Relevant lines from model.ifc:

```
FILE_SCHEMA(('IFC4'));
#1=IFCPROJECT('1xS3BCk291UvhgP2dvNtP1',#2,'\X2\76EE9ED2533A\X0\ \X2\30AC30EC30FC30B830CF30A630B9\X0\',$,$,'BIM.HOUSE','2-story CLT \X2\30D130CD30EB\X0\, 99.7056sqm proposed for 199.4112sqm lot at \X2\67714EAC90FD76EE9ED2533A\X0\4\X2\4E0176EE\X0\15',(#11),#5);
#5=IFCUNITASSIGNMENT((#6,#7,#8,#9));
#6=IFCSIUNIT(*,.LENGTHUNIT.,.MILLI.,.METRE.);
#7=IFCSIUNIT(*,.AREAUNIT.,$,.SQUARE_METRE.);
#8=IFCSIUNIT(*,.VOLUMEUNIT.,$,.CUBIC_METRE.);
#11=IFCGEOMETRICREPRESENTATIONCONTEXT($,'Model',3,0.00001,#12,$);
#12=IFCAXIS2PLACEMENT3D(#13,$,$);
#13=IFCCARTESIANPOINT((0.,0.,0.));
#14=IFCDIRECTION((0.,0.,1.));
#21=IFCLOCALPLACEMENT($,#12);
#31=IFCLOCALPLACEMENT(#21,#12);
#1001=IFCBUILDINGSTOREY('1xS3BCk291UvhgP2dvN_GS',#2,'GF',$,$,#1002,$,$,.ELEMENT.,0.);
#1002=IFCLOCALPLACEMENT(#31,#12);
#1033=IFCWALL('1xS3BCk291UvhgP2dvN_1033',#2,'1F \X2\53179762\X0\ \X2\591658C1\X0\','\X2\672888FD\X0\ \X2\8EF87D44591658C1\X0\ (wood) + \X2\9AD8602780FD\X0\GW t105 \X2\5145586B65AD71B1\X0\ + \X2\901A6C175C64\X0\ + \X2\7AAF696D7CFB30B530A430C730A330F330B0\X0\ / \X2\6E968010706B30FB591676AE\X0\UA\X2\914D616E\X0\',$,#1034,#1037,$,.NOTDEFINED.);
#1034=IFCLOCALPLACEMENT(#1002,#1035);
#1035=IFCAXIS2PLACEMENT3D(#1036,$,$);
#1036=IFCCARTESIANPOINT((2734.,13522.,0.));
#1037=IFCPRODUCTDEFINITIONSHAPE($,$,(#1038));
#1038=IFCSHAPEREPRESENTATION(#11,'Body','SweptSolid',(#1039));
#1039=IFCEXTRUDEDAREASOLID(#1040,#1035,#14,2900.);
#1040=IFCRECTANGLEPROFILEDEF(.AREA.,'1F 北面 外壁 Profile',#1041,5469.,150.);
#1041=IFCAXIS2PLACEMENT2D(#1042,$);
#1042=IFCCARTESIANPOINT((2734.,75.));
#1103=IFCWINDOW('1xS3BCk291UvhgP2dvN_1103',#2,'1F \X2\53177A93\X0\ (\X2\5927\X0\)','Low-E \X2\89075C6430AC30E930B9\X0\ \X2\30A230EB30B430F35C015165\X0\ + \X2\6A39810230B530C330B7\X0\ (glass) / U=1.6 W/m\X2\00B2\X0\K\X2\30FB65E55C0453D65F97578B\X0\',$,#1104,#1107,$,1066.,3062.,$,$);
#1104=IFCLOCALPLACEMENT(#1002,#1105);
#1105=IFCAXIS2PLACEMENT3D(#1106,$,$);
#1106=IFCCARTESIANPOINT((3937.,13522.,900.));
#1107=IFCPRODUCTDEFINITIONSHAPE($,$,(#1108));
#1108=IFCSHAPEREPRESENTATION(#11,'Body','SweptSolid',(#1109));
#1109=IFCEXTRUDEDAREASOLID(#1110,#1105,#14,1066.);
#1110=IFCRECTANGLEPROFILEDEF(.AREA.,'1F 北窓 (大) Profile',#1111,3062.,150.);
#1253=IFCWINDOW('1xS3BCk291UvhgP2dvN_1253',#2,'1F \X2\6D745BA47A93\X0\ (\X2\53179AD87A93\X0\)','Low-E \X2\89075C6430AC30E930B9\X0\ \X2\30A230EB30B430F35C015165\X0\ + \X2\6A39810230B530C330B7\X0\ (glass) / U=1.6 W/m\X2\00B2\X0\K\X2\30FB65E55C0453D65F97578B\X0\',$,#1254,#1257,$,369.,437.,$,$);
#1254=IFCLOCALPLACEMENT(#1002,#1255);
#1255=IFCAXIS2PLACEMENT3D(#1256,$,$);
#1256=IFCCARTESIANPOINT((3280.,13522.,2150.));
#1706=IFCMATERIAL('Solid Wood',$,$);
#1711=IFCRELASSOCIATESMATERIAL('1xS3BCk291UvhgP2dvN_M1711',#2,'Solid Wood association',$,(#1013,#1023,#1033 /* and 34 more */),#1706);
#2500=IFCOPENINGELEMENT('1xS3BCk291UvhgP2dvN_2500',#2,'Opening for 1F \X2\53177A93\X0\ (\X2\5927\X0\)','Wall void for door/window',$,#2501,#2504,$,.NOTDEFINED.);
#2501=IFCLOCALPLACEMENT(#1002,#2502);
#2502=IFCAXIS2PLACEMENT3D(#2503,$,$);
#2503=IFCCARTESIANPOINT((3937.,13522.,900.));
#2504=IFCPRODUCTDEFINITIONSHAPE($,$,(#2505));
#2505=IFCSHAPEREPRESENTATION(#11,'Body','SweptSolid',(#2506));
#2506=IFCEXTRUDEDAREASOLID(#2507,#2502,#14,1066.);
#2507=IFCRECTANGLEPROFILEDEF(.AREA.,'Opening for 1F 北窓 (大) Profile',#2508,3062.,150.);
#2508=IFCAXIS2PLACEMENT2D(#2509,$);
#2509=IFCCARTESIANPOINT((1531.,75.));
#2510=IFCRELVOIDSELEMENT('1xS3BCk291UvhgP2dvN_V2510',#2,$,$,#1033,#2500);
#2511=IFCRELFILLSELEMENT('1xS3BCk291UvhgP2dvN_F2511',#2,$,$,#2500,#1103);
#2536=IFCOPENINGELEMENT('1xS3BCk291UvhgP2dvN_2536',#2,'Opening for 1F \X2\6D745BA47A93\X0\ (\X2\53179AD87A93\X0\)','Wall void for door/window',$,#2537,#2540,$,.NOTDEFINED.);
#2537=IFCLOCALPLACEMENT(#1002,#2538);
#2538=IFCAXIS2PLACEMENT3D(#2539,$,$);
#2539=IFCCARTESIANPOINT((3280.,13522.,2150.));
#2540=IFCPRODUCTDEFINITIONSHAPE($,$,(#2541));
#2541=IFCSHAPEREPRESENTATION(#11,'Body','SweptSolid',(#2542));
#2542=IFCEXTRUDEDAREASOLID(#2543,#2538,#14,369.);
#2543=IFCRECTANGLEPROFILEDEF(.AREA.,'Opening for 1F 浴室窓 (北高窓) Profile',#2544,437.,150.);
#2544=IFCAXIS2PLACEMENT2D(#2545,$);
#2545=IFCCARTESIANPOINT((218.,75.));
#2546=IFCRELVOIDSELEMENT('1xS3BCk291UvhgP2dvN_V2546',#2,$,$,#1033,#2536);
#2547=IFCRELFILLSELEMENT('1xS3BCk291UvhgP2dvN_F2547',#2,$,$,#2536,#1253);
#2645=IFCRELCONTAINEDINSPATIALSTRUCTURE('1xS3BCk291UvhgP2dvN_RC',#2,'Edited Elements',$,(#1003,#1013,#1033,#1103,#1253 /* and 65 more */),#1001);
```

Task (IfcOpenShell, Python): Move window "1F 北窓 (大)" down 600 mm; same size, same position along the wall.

```python
import numpy as np
import ifcopenshell
import ifcopenshell.api.geometry
import ifcopenshell.util.placement
import ifcopenshell.util.unit

model = ifcopenshell.open("model.ifc")
unit_scale = ifcopenshell.util.unit.calculate_unit_scale(model)

window = model.by_guid("1xS3BCk291UvhgP2dvN_1103")
opening = window.FillsVoids[0].RelatingOpeningElement
dz = -600.0

shift = np.array([0.0, 0.0, dz])
# The window is not placed relative to its opening, so move both.
for product in (opening, window):
    matrix = ifcopenshell.util.placement.get_local_placement(product.ObjectPlacement)
    matrix[:3, 3] += shift
    ifcopenshell.api.geometry.edit_object_placement(model, product=product, matrix=matrix, is_si=False)

print(f"moved by {dz * unit_scale:+.3f} m")

model.write("model-out.ifc")
```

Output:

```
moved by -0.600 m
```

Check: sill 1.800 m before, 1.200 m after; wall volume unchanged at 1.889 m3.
